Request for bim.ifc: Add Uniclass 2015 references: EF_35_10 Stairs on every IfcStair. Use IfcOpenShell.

First a look at what the model holds.

```python
import ifcopenshell

model = ifcopenshell.open("bim.ifc")
print(model.schema)
print("classifications:", [c.Name for c in model.by_type("IfcClassification")])
for ifc_class in ("IfcDoor", "IfcRoof", "IfcStair", "IfcWall", "IfcWindow"):
    print(ifc_class, len(model.by_type(ifc_class)))
```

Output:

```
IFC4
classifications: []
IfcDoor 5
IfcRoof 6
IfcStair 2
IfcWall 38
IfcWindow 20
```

```python
import ifcopenshell
import ifcopenshell.api.classification

model = ifcopenshell.open("bim.ifc")

system = ifcopenshell.api.classification.add_classification(model, classification="Uniclass 2015")

codes = {
    "IfcStair": ("EF_35_10", "Stairs"),
}
for ifc_class, (code, name) in codes.items():
    products = model.by_type(ifc_class)
    ifcopenshell.api.classification.add_reference(
        model, products=products, classification=system, identification=code, name=name
    )
    print(code, len(products))

model.write("bim_v2.ifc")
```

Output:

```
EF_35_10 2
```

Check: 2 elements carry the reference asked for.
